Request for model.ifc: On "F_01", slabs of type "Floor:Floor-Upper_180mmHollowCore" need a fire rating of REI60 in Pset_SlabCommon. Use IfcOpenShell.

First a look at what the model holds.

```python
import ifcopenshell
import ifcopenshell.util.element

model = ifcopenshell.open("model.ifc")
print(model.schema)
storey = next(s for s in model.by_type("IfcBuildingStorey") if s.Name == "F_01")
slabs = [e for e in ifcopenshell.util.element.get_decomposition(storey) if e.is_a("IfcSlab")]
seen = {}
for e in slabs:
    element_type = ifcopenshell.util.element.get_type(e)
    key = (element_type.Name if element_type != e and element_type else None, ifcopenshell.util.element.get_pset(e, "Pset_SlabCommon", "FireRating"))
    seen[key] = seen.get(key, 0) + 1
for (name, value), count in sorted(seen.items(), key=str):
    print(count, "x", name, "|", value)
```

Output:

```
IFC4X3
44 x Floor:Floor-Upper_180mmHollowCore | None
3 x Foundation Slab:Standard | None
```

```python
import ifcopenshell
import ifcopenshell.api.pset
import ifcopenshell.util.element

model = ifcopenshell.open("model.ifc")

storey = next(s for s in model.by_type("IfcBuildingStorey") if s.Name == "F_01")
slabs = [e for e in ifcopenshell.util.element.get_decomposition(storey) if e.is_a("IfcSlab")]

count = 0
for e in slabs:
    element_type = ifcopenshell.util.element.get_type(e)
    if element_type in (None, e) or element_type.Name != "Floor:Floor-Upper_180mmHollowCore":
        continue
    # add_pset returns the element's existing set when there is one.
    pset = ifcopenshell.api.pset.add_pset(model, product=e, name="Pset_SlabCommon")
    ifcopenshell.api.pset.edit_pset(model, pset=pset, properties={"FireRating": "REI60"})
    count += 1

print(count, "slabs updated")

model.write("model_v2.ifc")
```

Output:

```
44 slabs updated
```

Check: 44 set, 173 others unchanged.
